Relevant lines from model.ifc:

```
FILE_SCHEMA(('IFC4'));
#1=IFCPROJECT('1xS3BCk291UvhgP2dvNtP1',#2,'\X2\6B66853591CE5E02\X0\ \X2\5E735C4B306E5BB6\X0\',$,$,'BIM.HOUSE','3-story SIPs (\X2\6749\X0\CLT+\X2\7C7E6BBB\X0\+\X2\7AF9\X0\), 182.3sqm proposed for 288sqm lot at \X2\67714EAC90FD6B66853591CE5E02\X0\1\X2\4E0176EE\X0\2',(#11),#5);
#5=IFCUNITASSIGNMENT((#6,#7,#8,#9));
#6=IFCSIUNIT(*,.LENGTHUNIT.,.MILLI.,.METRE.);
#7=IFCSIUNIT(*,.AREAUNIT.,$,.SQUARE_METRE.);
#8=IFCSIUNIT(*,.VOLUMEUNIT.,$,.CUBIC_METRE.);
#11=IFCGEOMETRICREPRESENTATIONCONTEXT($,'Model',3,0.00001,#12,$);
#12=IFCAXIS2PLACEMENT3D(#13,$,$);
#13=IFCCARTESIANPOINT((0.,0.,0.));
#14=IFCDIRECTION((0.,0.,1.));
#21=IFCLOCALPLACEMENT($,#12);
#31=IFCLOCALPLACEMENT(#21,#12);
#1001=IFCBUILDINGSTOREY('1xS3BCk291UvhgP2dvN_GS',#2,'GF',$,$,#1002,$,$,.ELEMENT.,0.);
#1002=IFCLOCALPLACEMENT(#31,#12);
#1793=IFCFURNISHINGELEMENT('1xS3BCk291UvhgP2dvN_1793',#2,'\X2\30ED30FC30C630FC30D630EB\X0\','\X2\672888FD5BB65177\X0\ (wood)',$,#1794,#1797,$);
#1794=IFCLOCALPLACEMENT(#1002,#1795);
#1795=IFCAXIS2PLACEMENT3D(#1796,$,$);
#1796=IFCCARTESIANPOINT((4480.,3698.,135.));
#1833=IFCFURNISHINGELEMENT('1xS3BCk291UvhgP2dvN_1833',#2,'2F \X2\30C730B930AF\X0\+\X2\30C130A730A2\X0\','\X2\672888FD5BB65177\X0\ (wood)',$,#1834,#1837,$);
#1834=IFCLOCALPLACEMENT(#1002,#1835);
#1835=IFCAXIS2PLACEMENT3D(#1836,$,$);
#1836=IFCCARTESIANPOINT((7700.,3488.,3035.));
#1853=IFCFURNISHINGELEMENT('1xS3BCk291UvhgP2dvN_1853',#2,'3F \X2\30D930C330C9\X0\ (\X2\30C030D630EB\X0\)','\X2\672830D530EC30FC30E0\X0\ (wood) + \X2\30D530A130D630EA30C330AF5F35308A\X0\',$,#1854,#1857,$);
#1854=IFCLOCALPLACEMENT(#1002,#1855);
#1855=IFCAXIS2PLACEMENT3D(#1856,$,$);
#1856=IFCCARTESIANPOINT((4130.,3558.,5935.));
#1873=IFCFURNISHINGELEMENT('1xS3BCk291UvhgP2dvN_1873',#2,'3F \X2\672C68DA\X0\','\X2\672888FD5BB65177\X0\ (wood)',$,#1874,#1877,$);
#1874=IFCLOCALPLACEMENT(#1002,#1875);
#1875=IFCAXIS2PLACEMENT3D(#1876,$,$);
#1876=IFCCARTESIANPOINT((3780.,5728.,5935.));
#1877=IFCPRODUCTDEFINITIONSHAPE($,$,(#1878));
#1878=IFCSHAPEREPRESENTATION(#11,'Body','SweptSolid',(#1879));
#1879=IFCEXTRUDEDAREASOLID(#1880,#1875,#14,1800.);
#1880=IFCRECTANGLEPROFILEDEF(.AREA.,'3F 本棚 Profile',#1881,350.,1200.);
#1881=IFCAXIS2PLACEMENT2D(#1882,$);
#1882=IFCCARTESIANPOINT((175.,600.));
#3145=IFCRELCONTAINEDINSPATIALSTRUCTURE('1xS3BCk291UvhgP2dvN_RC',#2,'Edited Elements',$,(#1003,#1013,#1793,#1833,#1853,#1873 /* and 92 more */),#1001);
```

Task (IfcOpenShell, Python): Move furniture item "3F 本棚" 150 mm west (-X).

```python
import ifcopenshell
import ifcopenshell.api.geometry
import ifcopenshell.util.placement

model = ifcopenshell.open("model.ifc")

item = model.by_guid("1xS3BCk291UvhgP2dvN_1873")
matrix = ifcopenshell.util.placement.get_local_placement(item.ObjectPlacement)
matrix[0, 3] -= 150.0
ifcopenshell.api.geometry.edit_object_placement(model, product=item, matrix=matrix, is_si=False)

print(ifcopenshell.util.placement.get_local_placement(item.ObjectPlacement).round(3) + 0.0)

model.write("model_rev.ifc")
```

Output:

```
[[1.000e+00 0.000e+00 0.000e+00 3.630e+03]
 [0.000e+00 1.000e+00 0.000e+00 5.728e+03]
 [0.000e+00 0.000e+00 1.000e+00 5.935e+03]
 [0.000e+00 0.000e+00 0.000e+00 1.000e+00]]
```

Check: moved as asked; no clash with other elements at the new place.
